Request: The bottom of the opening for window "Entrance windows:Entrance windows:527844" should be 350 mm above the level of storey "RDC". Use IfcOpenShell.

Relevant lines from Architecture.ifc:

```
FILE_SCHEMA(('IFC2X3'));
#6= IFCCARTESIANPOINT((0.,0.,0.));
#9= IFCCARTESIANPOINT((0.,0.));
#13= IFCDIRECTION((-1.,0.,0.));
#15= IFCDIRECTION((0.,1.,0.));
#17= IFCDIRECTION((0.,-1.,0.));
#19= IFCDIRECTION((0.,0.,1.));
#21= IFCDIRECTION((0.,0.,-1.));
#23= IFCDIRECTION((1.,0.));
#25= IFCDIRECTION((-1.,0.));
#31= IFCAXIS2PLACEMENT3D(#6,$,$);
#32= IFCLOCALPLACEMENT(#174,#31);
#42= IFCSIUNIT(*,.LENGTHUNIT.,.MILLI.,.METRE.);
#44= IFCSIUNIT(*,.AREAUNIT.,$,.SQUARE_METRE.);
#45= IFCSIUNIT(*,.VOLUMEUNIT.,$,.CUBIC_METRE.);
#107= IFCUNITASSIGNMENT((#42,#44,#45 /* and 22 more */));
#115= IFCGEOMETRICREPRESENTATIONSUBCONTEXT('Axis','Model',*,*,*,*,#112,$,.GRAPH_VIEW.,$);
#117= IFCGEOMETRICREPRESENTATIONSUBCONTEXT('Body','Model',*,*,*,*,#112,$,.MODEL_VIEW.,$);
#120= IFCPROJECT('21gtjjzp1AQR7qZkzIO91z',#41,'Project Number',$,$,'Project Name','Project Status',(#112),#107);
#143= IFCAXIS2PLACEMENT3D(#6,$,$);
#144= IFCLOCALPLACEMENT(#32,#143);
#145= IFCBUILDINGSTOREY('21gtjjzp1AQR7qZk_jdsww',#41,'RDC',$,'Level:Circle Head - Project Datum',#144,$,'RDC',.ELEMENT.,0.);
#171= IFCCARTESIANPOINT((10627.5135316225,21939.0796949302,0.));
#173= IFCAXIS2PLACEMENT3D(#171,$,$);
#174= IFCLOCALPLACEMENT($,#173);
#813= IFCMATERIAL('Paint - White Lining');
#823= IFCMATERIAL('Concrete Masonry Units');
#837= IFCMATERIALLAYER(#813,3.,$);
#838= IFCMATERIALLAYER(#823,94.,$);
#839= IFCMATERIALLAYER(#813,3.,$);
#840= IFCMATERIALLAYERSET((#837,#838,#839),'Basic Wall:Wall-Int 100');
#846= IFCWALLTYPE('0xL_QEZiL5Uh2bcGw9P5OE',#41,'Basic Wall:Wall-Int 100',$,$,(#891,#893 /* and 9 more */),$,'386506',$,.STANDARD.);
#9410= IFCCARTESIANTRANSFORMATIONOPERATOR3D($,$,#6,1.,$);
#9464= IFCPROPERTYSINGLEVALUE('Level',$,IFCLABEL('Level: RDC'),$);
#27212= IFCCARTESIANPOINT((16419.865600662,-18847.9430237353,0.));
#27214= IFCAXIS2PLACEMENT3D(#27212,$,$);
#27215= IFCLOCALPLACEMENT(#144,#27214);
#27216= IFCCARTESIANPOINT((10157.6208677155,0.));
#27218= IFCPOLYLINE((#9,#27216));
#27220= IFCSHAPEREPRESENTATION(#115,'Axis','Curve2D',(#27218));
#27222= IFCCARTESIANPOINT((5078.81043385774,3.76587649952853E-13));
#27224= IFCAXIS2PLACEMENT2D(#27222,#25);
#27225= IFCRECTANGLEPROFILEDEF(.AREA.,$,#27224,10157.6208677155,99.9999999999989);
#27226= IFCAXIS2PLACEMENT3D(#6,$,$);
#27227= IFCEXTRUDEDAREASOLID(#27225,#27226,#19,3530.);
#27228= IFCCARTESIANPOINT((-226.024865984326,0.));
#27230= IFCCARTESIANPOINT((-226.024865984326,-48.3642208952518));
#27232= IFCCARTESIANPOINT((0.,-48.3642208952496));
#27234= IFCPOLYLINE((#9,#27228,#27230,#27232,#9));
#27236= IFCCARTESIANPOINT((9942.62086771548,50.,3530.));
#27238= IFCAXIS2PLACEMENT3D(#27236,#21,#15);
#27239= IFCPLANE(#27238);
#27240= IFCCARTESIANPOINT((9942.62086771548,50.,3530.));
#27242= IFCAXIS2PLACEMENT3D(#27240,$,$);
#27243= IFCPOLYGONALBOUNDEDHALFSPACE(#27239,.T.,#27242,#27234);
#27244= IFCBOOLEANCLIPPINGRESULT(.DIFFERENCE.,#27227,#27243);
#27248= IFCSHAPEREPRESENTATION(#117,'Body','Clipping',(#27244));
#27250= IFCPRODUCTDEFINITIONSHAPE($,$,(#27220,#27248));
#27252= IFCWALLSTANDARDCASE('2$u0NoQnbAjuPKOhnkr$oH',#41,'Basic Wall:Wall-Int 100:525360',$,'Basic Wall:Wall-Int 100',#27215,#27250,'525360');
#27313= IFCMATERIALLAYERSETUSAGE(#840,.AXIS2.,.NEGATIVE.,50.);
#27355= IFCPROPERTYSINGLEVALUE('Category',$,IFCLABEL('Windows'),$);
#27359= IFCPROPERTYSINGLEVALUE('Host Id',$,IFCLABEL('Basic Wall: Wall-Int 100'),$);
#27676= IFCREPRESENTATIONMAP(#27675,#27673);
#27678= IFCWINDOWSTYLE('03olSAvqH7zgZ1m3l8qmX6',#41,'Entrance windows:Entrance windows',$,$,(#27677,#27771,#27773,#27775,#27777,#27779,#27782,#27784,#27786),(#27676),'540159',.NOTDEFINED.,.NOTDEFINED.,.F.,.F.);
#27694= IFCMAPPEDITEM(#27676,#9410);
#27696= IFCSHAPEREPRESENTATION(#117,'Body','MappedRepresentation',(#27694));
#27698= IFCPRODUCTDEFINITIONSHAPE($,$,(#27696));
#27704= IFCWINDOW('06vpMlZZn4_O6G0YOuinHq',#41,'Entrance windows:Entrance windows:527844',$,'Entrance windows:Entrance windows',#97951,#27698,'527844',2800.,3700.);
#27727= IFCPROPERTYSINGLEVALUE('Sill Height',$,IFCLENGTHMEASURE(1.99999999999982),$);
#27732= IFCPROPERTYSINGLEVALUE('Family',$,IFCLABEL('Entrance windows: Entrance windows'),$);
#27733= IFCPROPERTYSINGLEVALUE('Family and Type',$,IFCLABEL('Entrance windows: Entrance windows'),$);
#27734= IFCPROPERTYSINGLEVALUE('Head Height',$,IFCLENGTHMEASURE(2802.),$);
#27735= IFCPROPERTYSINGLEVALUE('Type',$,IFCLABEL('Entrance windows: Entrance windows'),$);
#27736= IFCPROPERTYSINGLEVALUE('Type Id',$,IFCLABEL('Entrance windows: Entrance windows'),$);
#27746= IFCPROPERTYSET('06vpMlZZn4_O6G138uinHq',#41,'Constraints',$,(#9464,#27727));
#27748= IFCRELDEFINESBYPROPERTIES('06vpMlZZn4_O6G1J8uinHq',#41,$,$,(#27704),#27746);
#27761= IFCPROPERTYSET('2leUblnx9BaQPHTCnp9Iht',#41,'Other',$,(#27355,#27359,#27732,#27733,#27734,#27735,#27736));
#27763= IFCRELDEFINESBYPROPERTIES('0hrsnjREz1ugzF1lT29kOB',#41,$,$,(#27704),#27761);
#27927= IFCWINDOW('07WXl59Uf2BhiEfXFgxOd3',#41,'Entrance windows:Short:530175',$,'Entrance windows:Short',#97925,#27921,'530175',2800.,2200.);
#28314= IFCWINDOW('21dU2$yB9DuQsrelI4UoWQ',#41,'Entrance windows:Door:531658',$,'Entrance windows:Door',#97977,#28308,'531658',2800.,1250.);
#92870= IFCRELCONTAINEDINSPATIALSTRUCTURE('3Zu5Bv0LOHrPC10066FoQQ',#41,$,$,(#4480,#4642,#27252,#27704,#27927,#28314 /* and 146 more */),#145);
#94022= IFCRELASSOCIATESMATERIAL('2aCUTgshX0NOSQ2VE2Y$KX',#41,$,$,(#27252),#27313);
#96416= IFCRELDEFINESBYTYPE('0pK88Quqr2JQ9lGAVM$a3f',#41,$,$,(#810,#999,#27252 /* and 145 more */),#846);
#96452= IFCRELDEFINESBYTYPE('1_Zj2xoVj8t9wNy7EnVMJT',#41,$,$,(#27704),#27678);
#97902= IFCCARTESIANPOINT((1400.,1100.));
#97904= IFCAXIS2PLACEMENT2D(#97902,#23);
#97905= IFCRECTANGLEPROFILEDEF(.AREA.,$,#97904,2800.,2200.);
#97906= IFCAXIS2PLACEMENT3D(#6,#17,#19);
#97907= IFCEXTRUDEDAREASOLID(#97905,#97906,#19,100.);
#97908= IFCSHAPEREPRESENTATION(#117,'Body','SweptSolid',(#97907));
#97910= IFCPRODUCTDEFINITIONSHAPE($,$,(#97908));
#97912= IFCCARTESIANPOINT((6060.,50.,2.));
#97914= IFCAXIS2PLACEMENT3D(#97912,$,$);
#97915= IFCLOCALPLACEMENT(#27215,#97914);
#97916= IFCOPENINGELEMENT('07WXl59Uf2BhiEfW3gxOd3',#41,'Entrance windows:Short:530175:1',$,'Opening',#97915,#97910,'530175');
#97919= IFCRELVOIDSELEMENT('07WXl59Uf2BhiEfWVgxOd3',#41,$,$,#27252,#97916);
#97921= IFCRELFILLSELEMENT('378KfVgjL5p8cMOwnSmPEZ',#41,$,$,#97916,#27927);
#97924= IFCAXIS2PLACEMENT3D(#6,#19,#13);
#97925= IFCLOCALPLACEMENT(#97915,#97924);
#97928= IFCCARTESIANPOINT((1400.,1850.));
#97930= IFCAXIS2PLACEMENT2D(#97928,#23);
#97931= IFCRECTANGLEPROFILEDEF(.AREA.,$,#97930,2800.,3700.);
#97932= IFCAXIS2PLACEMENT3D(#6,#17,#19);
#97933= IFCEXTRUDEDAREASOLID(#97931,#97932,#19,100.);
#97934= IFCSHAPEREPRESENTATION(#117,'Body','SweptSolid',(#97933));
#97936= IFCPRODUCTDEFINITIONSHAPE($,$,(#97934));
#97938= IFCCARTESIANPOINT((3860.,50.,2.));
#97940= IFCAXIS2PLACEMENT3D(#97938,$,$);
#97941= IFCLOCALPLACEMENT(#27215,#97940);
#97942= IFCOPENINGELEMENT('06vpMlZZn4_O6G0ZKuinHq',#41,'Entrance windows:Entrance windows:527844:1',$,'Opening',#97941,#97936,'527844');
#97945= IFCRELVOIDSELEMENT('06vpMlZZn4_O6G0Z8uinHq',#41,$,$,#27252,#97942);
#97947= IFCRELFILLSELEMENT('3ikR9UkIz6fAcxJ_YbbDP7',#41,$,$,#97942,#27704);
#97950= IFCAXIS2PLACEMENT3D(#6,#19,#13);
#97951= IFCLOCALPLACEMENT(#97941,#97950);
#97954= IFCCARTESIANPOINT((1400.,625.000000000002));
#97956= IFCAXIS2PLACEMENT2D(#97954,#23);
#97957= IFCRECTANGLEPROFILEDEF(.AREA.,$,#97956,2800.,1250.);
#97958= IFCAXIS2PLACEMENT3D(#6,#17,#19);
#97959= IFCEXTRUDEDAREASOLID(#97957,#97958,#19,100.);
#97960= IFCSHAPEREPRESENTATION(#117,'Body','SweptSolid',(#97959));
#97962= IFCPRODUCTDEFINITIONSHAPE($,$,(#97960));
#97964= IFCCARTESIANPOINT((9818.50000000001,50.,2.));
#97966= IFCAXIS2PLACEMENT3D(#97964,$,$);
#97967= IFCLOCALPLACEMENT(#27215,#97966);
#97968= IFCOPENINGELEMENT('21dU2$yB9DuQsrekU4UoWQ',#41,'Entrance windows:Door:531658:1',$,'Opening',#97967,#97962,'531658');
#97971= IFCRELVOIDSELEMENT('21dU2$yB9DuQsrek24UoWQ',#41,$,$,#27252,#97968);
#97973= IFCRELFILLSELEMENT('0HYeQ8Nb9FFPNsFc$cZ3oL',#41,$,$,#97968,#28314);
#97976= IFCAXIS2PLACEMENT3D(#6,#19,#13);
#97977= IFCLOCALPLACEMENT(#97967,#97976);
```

```python
import numpy as np
import ifcopenshell
import ifcopenshell.api.geometry
import ifcopenshell.api.pset
import ifcopenshell.geom
import ifcopenshell.util.element
import ifcopenshell.util.placement
import ifcopenshell.util.shape
import ifcopenshell.util.unit

model = ifcopenshell.open("Architecture.ifc")
unit_scale = ifcopenshell.util.unit.calculate_unit_scale(model)

window = model.by_guid("06vpMlZZn4_O6G0YOuinHq")
opening = window.FillsVoids[0].RelatingOpeningElement
storey = ifcopenshell.util.element.get_container(window, ifc_class="IfcBuildingStorey")
level = ifcopenshell.util.placement.get_local_placement(storey.ObjectPlacement)[2, 3]

# The opening's origin need not be at the sill, so measure its lowest point.
shape = ifcopenshell.geom.create_shape(ifcopenshell.geom.settings(), opening)
bottom = ifcopenshell.util.shape.get_shape_bottom_elevation(shape, shape.geometry) / unit_scale
dz = level + 350.0 - bottom

shift = np.array([0.0, 0.0, dz])
# The window is placed relative to its opening, so it follows when the opening moves.
matrix = ifcopenshell.util.placement.get_local_placement(opening.ObjectPlacement)
matrix[:3, 3] += shift
ifcopenshell.api.geometry.edit_object_placement(
    model, product=opening, matrix=matrix, is_si=False, should_transform_children=True
)

# Keep the stored heights in step.
pset = model.by_id(ifcopenshell.util.element.get_pset(window, "Constraints", should_inherit=False)["id"])
ifcopenshell.api.pset.edit_pset(model, pset=pset, properties={
    "Sill Height": model.create_entity("IfcLengthMeasure", ifcopenshell.util.element.get_pset(window, "Constraints", "Sill Height") + dz),
})
pset = model.by_id(ifcopenshell.util.element.get_pset(window, "Other", should_inherit=False)["id"])
ifcopenshell.api.pset.edit_pset(model, pset=pset, properties={
    "Head Height": model.create_entity("IfcLengthMeasure", ifcopenshell.util.element.get_pset(window, "Other", "Head Height") + dz),
})

print(f"moved by {dz * unit_scale:+.3f} m")

model.write("Architecture-out.ifc")
```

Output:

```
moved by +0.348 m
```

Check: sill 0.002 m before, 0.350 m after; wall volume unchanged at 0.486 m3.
